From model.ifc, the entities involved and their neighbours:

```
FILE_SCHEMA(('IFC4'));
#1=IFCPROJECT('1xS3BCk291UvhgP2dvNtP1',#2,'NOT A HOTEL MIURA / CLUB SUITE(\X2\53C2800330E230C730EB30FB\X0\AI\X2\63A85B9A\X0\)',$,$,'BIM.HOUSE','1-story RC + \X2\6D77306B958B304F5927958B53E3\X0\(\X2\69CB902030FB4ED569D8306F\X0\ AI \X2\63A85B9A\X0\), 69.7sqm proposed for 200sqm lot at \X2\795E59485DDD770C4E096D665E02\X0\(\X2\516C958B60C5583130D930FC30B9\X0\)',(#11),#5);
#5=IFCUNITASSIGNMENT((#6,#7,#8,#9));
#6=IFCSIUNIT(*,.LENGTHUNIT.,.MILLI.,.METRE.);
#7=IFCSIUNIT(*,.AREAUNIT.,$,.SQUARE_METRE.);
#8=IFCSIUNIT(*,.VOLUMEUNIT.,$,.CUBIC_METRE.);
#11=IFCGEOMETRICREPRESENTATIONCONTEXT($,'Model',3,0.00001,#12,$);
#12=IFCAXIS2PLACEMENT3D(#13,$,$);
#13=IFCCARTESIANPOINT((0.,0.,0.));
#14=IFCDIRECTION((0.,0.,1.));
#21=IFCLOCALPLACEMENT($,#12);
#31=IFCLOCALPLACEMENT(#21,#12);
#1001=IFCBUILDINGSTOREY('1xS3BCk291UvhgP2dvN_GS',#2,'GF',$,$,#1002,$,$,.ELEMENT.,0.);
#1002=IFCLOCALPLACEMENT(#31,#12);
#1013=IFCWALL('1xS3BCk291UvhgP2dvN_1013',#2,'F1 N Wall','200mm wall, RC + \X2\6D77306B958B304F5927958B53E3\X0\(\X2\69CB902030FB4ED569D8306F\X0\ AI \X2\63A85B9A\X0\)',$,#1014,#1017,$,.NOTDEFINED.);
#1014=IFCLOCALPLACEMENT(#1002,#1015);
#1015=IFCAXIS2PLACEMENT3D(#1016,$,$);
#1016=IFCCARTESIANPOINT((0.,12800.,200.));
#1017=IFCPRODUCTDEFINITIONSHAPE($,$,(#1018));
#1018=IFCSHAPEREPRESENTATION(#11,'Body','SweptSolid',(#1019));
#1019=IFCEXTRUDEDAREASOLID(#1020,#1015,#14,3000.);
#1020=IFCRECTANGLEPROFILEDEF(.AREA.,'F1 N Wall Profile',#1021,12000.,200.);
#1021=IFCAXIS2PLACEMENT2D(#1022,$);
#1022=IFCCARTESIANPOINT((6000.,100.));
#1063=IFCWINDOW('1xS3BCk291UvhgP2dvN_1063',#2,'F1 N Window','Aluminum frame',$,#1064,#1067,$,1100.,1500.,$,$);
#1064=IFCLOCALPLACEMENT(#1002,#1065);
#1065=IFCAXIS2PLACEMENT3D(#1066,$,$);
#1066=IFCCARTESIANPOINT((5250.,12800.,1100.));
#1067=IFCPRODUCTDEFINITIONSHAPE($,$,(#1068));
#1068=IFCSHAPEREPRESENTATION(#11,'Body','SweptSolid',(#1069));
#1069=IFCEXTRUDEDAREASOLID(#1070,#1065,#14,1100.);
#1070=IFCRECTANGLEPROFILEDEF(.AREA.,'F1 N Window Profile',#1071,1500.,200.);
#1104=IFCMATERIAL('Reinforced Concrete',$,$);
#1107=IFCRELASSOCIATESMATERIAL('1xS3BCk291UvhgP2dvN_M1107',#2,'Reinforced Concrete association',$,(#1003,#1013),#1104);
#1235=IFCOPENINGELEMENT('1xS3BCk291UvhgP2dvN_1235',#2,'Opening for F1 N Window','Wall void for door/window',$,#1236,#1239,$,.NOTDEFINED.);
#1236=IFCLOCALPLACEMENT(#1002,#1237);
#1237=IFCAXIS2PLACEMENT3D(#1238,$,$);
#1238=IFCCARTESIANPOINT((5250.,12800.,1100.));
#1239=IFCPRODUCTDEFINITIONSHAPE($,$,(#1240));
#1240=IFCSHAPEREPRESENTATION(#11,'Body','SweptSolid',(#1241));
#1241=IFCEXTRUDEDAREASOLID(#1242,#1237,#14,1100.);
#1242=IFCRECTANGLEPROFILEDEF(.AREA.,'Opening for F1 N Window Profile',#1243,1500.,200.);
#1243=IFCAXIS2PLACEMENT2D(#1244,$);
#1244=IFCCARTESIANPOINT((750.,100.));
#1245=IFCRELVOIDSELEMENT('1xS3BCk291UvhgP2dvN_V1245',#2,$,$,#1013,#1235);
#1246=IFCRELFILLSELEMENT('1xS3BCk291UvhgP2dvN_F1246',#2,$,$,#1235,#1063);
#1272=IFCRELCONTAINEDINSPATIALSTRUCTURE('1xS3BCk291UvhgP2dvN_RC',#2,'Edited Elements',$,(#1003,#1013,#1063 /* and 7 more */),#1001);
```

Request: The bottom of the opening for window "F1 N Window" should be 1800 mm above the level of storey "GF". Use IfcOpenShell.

```python
import numpy as np
import ifcopenshell
import ifcopenshell.api.geometry
import ifcopenshell.geom
import ifcopenshell.util.element
import ifcopenshell.util.placement
import ifcopenshell.util.shape
import ifcopenshell.util.unit

model = ifcopenshell.open("model.ifc")
unit_scale = ifcopenshell.util.unit.calculate_unit_scale(model)

window = model.by_id(1063)
opening = window.FillsVoids[0].RelatingOpeningElement
storey = ifcopenshell.util.element.get_container(window, ifc_class="IfcBuildingStorey")
level = ifcopenshell.util.placement.get_local_placement(storey.ObjectPlacement)[2, 3]

# The opening's origin need not be at the sill, so measure its lowest point.
shape = ifcopenshell.geom.create_shape(ifcopenshell.geom.settings(), opening)
bottom = ifcopenshell.util.shape.get_shape_bottom_elevation(shape, shape.geometry) / unit_scale
dz = level + 1800.0 - bottom

shift = np.array([0.0, 0.0, dz])
# The window is not placed relative to its opening, so move both.
for product in (opening, window):
    matrix = ifcopenshell.util.placement.get_local_placement(product.ObjectPlacement)
    matrix[:3, 3] += shift
    ifcopenshell.api.geometry.edit_object_placement(model, product=product, matrix=matrix, is_si=False)

print(f"moved by {dz * unit_scale:+.3f} m")

model.write("model_updated.ifc")
```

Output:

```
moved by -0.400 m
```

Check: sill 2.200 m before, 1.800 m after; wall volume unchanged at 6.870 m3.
